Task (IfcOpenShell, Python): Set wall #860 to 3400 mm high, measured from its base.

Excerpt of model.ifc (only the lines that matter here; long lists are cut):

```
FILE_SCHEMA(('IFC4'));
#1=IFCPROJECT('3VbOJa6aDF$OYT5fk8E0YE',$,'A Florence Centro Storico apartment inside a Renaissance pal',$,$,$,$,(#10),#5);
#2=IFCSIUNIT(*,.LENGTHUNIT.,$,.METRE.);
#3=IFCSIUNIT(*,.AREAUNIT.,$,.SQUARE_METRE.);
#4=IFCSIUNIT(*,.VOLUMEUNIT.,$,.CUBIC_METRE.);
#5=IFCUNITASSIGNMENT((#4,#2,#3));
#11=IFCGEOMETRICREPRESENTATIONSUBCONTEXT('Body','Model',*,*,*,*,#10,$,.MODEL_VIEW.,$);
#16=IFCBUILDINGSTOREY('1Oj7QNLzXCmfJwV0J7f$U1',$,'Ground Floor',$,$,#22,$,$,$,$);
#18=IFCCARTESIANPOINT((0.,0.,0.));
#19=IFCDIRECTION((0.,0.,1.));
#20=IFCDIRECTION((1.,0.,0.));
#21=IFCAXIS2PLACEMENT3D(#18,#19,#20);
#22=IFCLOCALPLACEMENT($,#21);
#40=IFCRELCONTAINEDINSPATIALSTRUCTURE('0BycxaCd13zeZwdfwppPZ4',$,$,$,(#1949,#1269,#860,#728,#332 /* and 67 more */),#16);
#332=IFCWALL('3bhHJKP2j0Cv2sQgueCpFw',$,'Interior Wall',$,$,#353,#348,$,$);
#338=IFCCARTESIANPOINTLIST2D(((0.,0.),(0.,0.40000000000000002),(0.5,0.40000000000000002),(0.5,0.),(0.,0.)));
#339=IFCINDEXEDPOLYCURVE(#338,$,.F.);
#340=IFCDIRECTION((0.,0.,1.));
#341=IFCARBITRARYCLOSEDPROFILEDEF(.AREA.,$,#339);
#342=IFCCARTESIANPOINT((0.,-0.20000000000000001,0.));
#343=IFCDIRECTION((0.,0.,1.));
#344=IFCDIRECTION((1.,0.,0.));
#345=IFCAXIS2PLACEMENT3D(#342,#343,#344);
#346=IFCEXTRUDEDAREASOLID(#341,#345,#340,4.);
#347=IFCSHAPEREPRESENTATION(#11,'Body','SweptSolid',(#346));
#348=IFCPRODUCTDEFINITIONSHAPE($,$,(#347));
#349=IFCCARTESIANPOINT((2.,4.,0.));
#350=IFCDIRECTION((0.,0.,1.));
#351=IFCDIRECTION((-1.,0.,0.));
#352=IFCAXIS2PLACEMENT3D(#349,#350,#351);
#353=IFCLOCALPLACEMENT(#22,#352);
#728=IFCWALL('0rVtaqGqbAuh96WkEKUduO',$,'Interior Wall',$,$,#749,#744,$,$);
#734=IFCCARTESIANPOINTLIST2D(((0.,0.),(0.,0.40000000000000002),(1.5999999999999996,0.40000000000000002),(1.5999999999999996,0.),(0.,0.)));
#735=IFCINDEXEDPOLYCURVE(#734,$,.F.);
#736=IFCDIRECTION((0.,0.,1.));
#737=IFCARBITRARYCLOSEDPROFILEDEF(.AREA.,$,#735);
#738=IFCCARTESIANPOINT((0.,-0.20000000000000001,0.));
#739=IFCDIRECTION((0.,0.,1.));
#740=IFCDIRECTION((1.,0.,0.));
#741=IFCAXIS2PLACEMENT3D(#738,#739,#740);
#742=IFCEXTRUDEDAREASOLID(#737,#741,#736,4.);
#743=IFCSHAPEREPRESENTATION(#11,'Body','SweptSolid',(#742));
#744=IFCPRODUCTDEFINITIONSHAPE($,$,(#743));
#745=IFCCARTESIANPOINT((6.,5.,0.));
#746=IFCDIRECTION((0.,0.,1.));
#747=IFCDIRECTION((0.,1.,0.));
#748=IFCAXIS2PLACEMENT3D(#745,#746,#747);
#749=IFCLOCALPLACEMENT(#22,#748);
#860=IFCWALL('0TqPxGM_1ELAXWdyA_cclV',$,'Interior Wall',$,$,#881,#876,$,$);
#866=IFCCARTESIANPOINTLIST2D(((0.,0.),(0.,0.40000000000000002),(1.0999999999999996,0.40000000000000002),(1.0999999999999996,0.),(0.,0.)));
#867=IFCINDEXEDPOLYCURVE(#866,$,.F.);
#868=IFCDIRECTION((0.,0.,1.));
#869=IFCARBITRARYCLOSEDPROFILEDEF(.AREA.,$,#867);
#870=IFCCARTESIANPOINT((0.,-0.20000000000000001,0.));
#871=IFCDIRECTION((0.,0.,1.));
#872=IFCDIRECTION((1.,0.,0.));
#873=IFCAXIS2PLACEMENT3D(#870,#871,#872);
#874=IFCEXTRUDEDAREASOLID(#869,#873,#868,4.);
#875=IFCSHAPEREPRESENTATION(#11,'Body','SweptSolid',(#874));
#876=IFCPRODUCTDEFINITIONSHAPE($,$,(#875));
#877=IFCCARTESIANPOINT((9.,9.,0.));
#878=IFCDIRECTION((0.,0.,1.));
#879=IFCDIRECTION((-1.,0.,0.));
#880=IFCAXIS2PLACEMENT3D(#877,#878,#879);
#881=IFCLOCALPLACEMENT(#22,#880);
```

```python
import ifcopenshell
import ifcopenshell.geom
import ifcopenshell.util.representation
import ifcopenshell.util.shape
import ifcopenshell.util.unit

model = ifcopenshell.open("model.ifc")
unit_scale = ifcopenshell.util.unit.calculate_unit_scale(model)
settings = ifcopenshell.geom.settings()


def volume(element):
    """Net volume in cubic metres, openings subtracted."""
    shape = ifcopenshell.geom.create_shape(settings, element)
    return ifcopenshell.util.shape.get_volume(shape.geometry)


wall = model.by_id(860)
before = volume(wall)

body = ifcopenshell.util.representation.get_representation(wall, "Model", "Body")
solid = body.Items[0]
old_height = solid.Depth
solid.Depth = 3.4 / unit_scale
after = volume(wall)

print(f"height {old_height:g} -> {solid.Depth:g}, volume {before:.3f} -> {after:.3f} m3")

model.write("model-out.ifc")
```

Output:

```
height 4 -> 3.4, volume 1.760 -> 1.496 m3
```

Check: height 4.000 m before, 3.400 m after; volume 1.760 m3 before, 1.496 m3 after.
